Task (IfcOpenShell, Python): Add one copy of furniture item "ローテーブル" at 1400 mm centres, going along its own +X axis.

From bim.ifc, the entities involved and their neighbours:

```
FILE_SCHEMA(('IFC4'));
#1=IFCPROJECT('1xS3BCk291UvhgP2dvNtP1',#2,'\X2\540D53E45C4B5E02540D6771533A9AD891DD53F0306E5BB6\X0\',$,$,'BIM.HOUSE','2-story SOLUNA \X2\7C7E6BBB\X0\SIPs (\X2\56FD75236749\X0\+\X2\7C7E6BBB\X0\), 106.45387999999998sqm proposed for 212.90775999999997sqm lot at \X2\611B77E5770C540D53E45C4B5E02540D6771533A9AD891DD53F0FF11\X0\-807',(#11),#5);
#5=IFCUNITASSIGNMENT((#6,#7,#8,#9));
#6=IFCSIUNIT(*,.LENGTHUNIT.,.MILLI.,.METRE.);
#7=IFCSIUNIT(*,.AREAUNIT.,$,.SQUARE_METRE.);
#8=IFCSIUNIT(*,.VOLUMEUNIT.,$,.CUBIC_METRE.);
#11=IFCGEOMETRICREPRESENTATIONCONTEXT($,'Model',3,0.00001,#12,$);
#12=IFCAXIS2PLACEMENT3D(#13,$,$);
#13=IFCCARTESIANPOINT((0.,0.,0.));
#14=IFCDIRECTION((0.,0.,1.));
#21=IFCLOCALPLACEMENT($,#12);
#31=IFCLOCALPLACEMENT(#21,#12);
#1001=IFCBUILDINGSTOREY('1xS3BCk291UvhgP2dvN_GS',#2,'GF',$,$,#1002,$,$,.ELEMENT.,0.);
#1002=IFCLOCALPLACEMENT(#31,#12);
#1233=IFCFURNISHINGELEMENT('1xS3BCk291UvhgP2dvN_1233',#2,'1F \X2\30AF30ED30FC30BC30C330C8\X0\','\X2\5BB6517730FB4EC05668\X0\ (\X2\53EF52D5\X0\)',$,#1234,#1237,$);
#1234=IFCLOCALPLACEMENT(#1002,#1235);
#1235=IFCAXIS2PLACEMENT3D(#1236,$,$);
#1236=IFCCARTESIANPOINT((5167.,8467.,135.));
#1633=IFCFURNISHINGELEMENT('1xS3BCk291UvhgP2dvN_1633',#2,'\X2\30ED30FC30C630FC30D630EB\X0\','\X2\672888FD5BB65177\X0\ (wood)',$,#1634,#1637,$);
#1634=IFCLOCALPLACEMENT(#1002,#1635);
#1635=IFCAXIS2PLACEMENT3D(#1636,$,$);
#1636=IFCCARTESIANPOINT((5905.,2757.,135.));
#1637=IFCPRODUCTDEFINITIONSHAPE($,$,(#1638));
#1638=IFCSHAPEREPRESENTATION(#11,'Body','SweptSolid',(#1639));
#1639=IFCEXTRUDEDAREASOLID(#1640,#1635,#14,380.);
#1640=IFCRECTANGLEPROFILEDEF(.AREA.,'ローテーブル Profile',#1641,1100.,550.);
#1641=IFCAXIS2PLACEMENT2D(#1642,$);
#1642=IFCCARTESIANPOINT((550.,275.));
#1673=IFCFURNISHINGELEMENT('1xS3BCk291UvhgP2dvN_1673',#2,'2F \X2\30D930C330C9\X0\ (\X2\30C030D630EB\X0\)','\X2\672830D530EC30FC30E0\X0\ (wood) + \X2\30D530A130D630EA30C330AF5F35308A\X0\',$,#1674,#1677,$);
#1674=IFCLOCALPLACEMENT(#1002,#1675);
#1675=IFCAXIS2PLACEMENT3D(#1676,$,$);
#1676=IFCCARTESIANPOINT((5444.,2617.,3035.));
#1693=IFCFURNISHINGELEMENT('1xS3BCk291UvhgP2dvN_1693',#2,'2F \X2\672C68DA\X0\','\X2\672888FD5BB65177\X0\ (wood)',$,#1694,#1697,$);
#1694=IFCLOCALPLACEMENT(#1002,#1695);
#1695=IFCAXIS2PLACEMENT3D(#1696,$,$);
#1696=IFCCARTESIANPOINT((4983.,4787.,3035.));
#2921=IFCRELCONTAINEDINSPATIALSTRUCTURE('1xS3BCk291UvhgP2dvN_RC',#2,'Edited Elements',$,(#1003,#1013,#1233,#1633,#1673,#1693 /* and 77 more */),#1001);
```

```python
import ifcopenshell
import ifcopenshell.api.geometry
import ifcopenshell.api.root
import ifcopenshell.util.element
import ifcopenshell.util.placement

model = ifcopenshell.open("bim.ifc")


def reuse_history(source, copy):
    """copy_class also copies each property set's owner history, people and application; keep the originals."""
    for rel in copy.IsDefinedBy:
        if rel.is_a("IfcRelDefinesByProperties") and (history := rel.RelatingPropertyDefinition.OwnerHistory):
            rel.RelatingPropertyDefinition.OwnerHistory = source.OwnerHistory
            ifcopenshell.util.element.remove_deep2(model, history)


source = model.by_guid("1xS3BCk291UvhgP2dvN_1633")
base = ifcopenshell.util.placement.get_local_placement(source.ObjectPlacement)
step = base[:3, 0] * 1400.0

for i in range(1, 2):
    copy = ifcopenshell.api.root.copy_class(model, product=source)
    copy.Representation = ifcopenshell.util.element.copy_deep(
        model, source.Representation, exclude=["IfcGeometricRepresentationContext", "IfcRepresentationMap"]
    )
    reuse_history(source, copy)
    matrix = base.copy()
    matrix[:3, 3] += i * step
    print("added at", matrix[:3, 3].round(3) + 0.0)
    ifcopenshell.api.geometry.edit_object_placement(model, product=copy, matrix=matrix, is_si=False)

model.write("bim-out.ifc")
```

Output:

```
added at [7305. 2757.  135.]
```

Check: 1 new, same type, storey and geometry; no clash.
